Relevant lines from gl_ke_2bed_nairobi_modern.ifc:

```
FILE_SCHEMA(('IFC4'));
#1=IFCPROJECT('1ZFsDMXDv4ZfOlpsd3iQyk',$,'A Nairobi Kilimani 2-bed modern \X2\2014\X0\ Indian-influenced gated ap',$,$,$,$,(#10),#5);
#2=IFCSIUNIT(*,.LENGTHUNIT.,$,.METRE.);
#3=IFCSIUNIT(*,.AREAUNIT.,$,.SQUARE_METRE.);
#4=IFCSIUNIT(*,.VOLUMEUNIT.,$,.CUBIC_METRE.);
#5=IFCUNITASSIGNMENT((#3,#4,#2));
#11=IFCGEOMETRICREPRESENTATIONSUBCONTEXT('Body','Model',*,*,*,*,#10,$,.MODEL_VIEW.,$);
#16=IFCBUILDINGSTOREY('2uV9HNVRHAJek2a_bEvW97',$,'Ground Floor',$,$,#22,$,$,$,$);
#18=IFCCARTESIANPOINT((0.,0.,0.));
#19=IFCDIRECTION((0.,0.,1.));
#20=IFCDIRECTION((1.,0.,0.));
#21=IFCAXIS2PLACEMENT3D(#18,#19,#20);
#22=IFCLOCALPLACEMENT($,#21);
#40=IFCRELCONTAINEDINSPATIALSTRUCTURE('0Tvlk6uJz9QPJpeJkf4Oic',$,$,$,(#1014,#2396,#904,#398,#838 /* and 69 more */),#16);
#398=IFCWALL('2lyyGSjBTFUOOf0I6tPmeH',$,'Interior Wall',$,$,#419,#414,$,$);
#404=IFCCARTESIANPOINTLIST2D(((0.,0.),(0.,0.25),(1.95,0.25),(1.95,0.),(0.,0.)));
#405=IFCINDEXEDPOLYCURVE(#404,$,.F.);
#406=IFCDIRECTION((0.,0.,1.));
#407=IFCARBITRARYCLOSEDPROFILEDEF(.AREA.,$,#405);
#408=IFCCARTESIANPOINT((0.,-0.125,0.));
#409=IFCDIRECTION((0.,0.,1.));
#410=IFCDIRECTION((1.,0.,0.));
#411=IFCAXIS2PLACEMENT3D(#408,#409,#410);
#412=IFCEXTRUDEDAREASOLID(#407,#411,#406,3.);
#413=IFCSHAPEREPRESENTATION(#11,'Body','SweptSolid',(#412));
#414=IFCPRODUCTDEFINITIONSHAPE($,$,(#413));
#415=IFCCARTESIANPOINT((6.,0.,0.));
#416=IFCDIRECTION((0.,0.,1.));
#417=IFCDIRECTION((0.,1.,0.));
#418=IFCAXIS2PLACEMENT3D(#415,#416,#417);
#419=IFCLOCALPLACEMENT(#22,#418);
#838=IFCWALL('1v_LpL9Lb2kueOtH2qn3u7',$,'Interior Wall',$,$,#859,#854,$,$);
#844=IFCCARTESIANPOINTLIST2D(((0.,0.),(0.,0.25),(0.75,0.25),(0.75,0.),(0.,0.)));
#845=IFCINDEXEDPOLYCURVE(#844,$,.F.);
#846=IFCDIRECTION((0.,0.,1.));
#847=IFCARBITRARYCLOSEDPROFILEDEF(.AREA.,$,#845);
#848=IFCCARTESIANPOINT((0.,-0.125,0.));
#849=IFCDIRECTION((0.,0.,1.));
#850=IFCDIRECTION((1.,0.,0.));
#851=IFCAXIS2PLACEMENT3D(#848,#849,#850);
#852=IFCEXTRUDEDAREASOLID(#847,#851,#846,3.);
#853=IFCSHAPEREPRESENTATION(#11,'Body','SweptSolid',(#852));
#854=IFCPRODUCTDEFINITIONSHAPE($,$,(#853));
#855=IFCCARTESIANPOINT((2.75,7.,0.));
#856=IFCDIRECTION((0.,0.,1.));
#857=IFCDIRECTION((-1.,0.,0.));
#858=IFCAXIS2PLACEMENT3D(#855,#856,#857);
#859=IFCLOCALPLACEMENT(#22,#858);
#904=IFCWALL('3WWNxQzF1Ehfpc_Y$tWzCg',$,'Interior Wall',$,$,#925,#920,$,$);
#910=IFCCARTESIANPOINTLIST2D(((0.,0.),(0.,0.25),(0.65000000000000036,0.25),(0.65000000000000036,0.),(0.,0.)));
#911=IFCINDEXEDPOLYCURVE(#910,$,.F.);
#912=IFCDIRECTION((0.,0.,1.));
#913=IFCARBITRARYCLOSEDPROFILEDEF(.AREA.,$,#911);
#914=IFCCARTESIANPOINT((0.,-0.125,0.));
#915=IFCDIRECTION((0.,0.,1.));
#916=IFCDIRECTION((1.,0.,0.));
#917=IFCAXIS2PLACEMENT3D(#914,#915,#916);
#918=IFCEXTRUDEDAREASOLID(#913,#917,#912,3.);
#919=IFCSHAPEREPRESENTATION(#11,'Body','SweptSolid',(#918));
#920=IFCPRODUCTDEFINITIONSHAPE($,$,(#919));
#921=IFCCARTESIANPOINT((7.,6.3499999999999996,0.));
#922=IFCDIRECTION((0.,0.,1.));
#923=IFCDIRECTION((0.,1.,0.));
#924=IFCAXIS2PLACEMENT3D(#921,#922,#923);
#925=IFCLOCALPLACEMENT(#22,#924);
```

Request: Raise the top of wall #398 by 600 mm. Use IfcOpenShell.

```python
import ifcopenshell
import ifcopenshell.geom
import ifcopenshell.util.representation
import ifcopenshell.util.shape

model = ifcopenshell.open("gl_ke_2bed_nairobi_modern.ifc")
settings = ifcopenshell.geom.settings()


def volume(element):
    """Net volume in cubic metres, openings subtracted."""
    shape = ifcopenshell.geom.create_shape(settings, element)
    return ifcopenshell.util.shape.get_volume(shape.geometry)


wall = model.by_guid("2lyyGSjBTFUOOf0I6tPmeH")
before = volume(wall)

body = ifcopenshell.util.representation.get_representation(wall, "Model", "Body")
solid = body.Items[0]
old_height = solid.Depth
solid.Depth += 0.6
after = volume(wall)

print(f"height {old_height:g} -> {solid.Depth:g}, volume {before:.3f} -> {after:.3f} m3")

model.write("gl_ke_2bed_nairobi_modern_v2.ifc")
```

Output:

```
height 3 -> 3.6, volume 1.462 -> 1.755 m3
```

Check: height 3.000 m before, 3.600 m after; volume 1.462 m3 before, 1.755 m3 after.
